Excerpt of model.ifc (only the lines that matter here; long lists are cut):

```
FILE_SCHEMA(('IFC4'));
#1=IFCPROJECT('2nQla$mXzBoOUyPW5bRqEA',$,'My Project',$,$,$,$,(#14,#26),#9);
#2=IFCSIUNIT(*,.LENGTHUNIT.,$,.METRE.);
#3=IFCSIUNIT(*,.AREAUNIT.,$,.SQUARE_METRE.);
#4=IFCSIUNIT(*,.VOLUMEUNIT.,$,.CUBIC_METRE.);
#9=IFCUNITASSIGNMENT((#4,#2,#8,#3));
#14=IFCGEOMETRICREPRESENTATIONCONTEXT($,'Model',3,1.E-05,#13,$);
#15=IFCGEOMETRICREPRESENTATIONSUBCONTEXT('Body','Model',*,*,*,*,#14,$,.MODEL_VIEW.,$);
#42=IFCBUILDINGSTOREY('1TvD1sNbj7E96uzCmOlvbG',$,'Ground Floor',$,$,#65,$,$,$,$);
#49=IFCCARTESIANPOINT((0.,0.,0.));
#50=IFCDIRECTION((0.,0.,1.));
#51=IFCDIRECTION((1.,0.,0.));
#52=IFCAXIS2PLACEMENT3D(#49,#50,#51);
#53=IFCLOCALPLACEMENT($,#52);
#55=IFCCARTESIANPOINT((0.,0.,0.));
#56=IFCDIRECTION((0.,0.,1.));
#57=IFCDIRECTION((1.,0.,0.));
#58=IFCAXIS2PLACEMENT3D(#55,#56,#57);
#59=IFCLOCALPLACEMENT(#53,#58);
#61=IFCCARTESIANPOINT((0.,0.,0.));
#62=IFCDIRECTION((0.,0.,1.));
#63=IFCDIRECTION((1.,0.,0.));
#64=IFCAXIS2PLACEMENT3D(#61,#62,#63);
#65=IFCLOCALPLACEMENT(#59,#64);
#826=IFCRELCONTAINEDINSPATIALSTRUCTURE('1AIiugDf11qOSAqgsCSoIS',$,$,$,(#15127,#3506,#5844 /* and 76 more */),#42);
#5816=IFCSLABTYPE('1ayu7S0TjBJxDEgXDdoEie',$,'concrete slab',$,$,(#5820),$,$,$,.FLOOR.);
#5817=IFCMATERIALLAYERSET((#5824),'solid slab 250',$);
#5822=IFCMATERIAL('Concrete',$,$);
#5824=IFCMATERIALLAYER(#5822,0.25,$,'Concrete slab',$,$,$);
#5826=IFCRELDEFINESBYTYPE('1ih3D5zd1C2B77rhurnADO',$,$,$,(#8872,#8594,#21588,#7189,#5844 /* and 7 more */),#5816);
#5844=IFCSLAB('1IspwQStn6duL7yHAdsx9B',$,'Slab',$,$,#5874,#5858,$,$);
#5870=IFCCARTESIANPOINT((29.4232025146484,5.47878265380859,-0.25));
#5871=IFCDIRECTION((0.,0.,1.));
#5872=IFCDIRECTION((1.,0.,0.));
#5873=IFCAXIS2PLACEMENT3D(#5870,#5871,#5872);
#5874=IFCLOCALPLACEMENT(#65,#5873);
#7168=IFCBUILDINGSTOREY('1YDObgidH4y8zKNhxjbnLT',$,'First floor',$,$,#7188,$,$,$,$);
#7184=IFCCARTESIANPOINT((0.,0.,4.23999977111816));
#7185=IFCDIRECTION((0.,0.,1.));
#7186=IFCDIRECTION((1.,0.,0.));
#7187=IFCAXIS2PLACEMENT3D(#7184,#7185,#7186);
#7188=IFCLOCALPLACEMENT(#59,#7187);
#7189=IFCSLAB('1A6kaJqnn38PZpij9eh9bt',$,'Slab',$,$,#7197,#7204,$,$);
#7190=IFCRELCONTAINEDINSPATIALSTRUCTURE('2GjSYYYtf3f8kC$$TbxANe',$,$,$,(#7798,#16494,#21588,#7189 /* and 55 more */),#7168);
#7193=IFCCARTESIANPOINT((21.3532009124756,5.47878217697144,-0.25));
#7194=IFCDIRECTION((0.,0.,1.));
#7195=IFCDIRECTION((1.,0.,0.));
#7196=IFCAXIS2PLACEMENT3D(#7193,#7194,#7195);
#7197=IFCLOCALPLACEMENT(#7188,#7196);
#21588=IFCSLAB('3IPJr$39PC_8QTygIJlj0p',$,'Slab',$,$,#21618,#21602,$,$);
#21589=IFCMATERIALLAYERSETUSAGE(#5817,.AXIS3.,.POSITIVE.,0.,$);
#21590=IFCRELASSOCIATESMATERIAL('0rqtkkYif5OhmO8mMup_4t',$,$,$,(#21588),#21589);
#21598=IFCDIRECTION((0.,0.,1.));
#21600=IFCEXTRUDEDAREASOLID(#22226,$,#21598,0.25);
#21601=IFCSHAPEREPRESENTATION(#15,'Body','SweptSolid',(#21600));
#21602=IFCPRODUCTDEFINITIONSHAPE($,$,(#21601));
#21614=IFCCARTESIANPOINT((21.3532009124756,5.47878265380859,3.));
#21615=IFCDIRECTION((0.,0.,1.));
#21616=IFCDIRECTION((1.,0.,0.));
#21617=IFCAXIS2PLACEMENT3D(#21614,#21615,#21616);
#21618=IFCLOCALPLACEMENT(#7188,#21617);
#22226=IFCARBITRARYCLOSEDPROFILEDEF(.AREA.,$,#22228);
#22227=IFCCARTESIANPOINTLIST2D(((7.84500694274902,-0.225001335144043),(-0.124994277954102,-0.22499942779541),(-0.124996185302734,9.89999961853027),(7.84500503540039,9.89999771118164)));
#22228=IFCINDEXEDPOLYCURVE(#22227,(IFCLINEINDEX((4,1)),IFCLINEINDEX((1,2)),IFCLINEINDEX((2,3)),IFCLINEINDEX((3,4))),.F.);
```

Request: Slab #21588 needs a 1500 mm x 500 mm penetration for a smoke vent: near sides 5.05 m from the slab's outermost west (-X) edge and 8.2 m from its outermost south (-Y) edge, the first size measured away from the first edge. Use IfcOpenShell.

```python
import numpy as np
import ifcopenshell
import ifcopenshell.api.feature
import ifcopenshell.api.geometry
import ifcopenshell.api.root
import ifcopenshell.geom
import ifcopenshell.util.placement
import ifcopenshell.util.representation
import ifcopenshell.util.shape
import ifcopenshell.util.unit

model = ifcopenshell.open("model.ifc")
unit_scale = ifcopenshell.util.unit.calculate_unit_scale(model)
settings = ifcopenshell.geom.settings()


def volume(element):
    """Net volume in cubic metres, openings subtracted."""
    shape = ifcopenshell.geom.create_shape(settings, element)
    return ifcopenshell.util.shape.get_volume(shape.geometry)


slab = model.by_id(21588)
before = volume(slab)

# Extent in the slab's own axes, in metres. The edges named are its -X and -Y sides.
slab_shape = ifcopenshell.geom.create_shape(settings, slab)
vertices = ifcopenshell.util.shape.get_vertices(slab_shape.geometry)
x_min, y_min, bottom = vertices.min(axis=0)
top = vertices[:, 2].max()

opening = ifcopenshell.api.root.create_entity(model, ifc_class="IfcOpeningElement", name="Smoke vent opening", predefined_type="OPENING")
context = ifcopenshell.util.representation.get_context(model, "Model", "Body", "MODEL_VIEW")
width, depth = 1.5, 0.5
outline = [(0.0, 0.0), (width, 0.0), (width, depth), (0.0, depth), (0.0, 0.0)]
# Overshoot both faces by 50 mm so the cut is clean.
shape = ifcopenshell.api.geometry.add_slab_representation(
    model, context=context, depth=top - bottom + 0.1, polyline=outline
)
ifcopenshell.api.geometry.assign_representation(model, product=opening, representation=shape)

matrix = ifcopenshell.util.placement.get_local_placement(slab.ObjectPlacement)
matrix[:, 3] = matrix @ np.append(np.array([x_min + 5.05, y_min + 8.2, bottom - 0.05]) / unit_scale, 1.0)
ifcopenshell.api.geometry.edit_object_placement(model, product=opening, matrix=matrix, is_si=False)
ifcopenshell.api.feature.add_feature(model, feature=opening, element=slab)

after = volume(slab)

print(f"slab volume {before:.3f} -> {after:.3f} m3")

model.write("model_v2.ifc")
```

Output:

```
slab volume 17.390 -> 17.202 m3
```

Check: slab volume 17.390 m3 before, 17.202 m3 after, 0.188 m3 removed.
